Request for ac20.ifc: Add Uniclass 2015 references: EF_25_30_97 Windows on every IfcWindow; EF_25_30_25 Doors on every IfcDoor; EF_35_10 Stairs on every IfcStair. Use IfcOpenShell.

First a look at what the model holds.

```python
import ifcopenshell

model = ifcopenshell.open("ac20.ifc")
print(model.schema)
print("classifications:", [c.Name for c in model.by_type("IfcClassification")])
for ifc_class in ("IfcDoor", "IfcRoof", "IfcStair", "IfcWall", "IfcWindow"):
    print(ifc_class, len(model.by_type(ifc_class)))
```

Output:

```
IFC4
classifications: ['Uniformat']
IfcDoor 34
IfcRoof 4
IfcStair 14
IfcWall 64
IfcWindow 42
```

```python
import ifcopenshell
import ifcopenshell.api.classification

model = ifcopenshell.open("ac20.ifc")

system = ifcopenshell.api.classification.add_classification(model, classification="Uniclass 2015")

codes = {
    "IfcWindow": ("EF_25_30_97", "Windows"),
    "IfcDoor": ("EF_25_30_25", "Doors"),
    "IfcStair": ("EF_35_10", "Stairs"),
}
for ifc_class, (code, name) in codes.items():
    products = model.by_type(ifc_class)
    ifcopenshell.api.classification.add_reference(
        model, products=products, classification=system, identification=code, name=name
    )
    print(code, len(products))

model.write("ac20_v2.ifc")
```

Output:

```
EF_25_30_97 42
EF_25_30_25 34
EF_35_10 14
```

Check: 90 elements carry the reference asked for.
